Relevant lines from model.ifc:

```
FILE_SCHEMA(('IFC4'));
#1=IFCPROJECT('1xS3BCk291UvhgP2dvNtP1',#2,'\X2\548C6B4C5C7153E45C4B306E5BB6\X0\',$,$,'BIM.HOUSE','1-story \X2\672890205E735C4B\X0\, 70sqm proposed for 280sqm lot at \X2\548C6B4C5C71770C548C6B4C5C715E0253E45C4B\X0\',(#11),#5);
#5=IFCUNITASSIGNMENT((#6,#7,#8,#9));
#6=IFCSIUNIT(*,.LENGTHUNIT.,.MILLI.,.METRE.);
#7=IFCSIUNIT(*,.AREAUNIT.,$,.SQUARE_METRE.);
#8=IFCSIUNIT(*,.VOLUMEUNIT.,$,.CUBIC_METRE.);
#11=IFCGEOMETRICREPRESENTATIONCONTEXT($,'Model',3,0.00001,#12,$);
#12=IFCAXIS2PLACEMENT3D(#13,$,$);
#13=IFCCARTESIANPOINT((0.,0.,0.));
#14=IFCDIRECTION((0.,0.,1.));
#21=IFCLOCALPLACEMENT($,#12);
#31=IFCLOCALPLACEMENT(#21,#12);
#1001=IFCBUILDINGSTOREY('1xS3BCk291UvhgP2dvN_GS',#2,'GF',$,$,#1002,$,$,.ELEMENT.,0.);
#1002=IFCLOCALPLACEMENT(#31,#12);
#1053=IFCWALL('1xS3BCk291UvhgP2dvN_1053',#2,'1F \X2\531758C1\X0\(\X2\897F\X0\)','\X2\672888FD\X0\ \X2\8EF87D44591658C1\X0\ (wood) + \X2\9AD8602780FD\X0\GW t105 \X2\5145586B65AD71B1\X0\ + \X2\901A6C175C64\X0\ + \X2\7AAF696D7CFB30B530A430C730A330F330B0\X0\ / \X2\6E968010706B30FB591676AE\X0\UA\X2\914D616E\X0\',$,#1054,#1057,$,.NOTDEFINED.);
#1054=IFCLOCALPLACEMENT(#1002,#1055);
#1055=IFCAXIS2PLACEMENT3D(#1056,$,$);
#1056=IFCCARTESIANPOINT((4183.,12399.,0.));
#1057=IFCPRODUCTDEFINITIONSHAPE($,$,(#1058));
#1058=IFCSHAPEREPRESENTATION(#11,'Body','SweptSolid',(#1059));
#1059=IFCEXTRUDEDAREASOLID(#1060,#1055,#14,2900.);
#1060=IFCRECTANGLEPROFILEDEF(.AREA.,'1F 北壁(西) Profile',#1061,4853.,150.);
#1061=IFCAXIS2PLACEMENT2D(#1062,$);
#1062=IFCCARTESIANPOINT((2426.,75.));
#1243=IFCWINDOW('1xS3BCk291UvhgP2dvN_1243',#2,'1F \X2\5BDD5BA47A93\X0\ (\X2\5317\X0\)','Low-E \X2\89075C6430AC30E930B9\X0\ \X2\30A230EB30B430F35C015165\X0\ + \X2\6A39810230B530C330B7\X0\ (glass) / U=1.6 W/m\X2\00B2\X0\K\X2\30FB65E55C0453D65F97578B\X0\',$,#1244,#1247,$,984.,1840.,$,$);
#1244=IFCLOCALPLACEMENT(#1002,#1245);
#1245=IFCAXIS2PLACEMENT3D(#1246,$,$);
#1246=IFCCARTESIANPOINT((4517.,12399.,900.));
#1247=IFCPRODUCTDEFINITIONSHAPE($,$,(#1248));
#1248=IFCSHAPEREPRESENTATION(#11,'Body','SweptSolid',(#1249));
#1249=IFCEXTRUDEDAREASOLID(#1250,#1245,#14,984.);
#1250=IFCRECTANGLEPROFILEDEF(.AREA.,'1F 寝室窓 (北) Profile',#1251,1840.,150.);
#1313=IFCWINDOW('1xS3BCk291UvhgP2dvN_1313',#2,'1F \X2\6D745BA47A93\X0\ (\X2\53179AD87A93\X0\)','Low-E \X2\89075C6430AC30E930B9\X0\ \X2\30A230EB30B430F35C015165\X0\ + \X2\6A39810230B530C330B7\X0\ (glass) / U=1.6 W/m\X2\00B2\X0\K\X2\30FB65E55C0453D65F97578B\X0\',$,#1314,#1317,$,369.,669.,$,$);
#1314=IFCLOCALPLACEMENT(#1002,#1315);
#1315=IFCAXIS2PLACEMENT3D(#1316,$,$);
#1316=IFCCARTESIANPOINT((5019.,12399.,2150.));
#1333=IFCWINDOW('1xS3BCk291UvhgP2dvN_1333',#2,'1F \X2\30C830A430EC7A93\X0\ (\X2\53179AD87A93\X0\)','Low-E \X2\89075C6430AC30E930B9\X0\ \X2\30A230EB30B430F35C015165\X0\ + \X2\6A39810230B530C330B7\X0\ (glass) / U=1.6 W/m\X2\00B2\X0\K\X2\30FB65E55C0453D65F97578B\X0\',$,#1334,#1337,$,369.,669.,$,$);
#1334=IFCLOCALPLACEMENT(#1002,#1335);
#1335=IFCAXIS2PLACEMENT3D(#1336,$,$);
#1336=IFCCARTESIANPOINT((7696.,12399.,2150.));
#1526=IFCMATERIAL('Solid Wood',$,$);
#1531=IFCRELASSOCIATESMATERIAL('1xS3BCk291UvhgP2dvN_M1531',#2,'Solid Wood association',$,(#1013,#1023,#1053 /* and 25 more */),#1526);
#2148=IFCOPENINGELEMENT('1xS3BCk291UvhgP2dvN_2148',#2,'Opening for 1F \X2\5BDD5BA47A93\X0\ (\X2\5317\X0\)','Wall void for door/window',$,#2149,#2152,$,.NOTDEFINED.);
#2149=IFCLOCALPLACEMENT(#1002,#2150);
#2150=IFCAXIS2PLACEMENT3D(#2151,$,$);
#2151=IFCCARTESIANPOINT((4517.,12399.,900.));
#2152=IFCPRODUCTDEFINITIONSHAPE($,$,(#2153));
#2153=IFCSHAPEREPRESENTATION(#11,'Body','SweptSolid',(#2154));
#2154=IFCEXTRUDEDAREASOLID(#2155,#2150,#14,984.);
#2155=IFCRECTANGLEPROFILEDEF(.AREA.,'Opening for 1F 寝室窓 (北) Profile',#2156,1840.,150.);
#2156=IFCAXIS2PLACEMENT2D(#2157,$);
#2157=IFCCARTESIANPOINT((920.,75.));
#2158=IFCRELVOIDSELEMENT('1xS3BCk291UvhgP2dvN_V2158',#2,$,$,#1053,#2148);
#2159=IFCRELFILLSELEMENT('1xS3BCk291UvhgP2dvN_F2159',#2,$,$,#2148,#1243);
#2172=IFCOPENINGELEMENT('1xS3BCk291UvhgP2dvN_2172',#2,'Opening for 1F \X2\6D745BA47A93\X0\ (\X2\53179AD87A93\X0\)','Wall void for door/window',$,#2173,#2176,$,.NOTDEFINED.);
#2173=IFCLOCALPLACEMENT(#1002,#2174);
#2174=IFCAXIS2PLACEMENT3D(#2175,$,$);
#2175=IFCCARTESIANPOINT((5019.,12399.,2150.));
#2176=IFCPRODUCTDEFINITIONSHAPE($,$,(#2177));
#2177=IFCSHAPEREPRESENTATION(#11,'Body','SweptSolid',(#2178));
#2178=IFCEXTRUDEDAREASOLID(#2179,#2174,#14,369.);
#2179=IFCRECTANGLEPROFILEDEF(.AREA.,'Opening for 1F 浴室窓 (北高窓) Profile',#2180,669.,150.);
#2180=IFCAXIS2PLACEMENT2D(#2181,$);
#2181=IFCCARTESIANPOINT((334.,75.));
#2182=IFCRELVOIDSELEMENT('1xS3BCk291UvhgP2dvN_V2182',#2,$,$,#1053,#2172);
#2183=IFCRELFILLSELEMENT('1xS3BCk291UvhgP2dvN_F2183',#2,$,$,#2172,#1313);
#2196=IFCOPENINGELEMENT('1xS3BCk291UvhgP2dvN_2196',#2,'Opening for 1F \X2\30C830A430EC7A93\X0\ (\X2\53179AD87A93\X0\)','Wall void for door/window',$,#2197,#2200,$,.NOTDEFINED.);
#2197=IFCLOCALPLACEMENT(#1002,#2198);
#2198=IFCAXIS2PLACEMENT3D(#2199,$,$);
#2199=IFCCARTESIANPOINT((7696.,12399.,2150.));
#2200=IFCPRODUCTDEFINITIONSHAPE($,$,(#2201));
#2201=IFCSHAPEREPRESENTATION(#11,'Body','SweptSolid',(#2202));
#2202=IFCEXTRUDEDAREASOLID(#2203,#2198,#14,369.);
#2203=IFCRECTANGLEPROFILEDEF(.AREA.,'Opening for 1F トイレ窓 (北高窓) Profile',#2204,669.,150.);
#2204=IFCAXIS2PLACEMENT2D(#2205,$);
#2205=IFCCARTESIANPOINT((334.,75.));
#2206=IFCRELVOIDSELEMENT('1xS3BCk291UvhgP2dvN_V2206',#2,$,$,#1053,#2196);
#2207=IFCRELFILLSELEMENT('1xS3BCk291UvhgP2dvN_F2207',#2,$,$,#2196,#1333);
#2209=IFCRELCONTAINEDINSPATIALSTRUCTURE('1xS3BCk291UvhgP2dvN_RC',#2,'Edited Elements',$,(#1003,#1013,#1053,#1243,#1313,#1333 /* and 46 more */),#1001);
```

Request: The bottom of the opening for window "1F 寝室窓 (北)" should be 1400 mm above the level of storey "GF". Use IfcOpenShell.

```python
import numpy as np
import ifcopenshell
import ifcopenshell.api.geometry
import ifcopenshell.geom
import ifcopenshell.util.element
import ifcopenshell.util.placement
import ifcopenshell.util.shape
import ifcopenshell.util.unit

model = ifcopenshell.open("model.ifc")
unit_scale = ifcopenshell.util.unit.calculate_unit_scale(model)

window = model.by_id(1243)
opening = window.FillsVoids[0].RelatingOpeningElement
storey = ifcopenshell.util.element.get_container(window, ifc_class="IfcBuildingStorey")
level = ifcopenshell.util.placement.get_local_placement(storey.ObjectPlacement)[2, 3]

# The opening's origin need not be at the sill, so measure its lowest point.
shape = ifcopenshell.geom.create_shape(ifcopenshell.geom.settings(), opening)
bottom = ifcopenshell.util.shape.get_shape_bottom_elevation(shape, shape.geometry) / unit_scale
dz = level + 1.4 / unit_scale - bottom

shift = np.array([0.0, 0.0, dz])
# The window is not placed relative to its opening, so move both.
for product in (opening, window):
    matrix = ifcopenshell.util.placement.get_local_placement(product.ObjectPlacement)
    matrix[:3, 3] += shift
    ifcopenshell.api.geometry.edit_object_placement(model, product=product, matrix=matrix, is_si=False)

print(f"moved by {dz * unit_scale:+.3f} m")

model.write("model_rev.ifc")
```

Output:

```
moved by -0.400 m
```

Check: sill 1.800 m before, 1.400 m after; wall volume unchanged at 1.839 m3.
